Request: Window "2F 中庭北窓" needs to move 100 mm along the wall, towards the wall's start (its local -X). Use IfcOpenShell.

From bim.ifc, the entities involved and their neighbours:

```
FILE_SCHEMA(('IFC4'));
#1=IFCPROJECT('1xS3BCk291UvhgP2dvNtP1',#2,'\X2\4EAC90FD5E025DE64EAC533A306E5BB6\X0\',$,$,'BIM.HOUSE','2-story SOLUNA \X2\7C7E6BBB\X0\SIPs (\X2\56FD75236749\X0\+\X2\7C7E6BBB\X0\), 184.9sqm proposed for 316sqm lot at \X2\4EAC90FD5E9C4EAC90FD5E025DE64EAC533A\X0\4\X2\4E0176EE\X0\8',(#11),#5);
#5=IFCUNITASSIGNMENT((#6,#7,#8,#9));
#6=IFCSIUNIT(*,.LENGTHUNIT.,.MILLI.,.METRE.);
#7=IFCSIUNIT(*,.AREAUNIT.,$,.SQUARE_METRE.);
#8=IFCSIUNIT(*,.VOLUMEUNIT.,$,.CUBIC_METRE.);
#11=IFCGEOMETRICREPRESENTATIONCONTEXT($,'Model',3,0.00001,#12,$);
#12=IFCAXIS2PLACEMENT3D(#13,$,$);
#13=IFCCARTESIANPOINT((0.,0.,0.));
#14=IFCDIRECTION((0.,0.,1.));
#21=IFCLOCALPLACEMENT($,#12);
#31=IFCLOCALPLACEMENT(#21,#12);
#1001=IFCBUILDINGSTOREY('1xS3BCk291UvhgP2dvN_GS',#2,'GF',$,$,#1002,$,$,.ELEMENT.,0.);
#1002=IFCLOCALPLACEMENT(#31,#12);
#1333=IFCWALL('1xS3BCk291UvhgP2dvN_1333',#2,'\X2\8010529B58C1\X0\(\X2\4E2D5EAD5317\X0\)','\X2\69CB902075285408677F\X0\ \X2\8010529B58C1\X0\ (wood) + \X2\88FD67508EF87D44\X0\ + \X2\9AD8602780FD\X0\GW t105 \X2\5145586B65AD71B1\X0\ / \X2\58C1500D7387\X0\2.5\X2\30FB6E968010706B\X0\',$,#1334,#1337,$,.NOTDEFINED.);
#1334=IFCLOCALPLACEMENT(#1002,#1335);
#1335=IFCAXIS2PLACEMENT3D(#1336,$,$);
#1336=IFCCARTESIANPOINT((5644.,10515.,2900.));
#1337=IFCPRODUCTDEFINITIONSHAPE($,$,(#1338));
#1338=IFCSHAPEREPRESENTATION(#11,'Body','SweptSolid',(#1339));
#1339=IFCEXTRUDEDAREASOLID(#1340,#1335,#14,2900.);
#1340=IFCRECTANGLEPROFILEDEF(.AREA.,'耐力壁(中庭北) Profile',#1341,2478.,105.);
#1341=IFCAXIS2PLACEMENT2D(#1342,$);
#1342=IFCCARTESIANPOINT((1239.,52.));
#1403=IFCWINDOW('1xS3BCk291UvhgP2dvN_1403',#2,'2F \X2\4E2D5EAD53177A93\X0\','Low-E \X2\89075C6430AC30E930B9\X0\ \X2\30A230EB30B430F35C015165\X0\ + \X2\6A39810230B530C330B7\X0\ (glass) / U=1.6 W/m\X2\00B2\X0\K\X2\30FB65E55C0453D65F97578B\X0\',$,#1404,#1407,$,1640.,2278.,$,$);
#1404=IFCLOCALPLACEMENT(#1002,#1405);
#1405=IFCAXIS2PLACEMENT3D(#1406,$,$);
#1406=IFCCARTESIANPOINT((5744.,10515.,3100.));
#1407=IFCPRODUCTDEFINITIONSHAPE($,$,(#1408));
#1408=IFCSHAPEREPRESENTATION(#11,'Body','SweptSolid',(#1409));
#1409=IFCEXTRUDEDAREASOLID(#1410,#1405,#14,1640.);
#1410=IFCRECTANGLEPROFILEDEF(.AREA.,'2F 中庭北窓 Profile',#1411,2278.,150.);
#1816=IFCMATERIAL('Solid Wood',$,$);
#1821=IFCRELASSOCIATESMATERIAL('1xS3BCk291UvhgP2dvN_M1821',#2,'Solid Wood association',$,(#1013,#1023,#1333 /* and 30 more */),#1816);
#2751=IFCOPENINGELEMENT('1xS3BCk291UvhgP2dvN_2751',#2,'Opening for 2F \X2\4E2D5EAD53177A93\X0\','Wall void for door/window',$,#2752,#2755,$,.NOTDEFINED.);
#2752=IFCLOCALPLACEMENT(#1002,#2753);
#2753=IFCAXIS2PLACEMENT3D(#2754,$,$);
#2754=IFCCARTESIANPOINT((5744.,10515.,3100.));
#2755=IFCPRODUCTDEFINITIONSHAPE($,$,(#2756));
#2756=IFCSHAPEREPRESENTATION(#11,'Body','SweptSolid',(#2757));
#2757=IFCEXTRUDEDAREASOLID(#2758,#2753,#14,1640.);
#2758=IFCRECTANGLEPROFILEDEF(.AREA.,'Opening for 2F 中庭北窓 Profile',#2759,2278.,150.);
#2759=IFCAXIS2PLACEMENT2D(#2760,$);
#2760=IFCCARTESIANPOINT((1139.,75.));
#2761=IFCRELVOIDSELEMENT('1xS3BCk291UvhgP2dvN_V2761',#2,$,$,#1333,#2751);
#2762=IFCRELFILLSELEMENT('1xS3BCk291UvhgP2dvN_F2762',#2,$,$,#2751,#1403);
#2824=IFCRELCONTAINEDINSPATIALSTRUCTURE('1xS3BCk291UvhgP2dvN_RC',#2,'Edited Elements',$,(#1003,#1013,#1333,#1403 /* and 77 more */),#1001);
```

```python
import ifcopenshell
import ifcopenshell.api.geometry
import ifcopenshell.util.placement

model = ifcopenshell.open("bim.ifc")

window = model.by_id(1403)
opening = window.FillsVoids[0].RelatingOpeningElement
wall = opening.VoidsElements[0].RelatingBuildingElement

wall_matrix = ifcopenshell.util.placement.get_local_placement(wall.ObjectPlacement)
shift = wall_matrix[:3, 0] * -100.0
before = ifcopenshell.util.placement.get_local_placement(window.ObjectPlacement)[:3, 3].copy()

# The window is not placed relative to its opening, so move both.
for product in (opening, window):
    matrix = ifcopenshell.util.placement.get_local_placement(product.ObjectPlacement)
    matrix[:3, 3] += shift
    ifcopenshell.api.geometry.edit_object_placement(model, product=product, matrix=matrix, is_si=False)

after = ifcopenshell.util.placement.get_local_placement(window.ObjectPlacement)[:3, 3]
print("window moved by", (after - before).round(3) + 0.0)

model.write("bim_rev.ifc")
```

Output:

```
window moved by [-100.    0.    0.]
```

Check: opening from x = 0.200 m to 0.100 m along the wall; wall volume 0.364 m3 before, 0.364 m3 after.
